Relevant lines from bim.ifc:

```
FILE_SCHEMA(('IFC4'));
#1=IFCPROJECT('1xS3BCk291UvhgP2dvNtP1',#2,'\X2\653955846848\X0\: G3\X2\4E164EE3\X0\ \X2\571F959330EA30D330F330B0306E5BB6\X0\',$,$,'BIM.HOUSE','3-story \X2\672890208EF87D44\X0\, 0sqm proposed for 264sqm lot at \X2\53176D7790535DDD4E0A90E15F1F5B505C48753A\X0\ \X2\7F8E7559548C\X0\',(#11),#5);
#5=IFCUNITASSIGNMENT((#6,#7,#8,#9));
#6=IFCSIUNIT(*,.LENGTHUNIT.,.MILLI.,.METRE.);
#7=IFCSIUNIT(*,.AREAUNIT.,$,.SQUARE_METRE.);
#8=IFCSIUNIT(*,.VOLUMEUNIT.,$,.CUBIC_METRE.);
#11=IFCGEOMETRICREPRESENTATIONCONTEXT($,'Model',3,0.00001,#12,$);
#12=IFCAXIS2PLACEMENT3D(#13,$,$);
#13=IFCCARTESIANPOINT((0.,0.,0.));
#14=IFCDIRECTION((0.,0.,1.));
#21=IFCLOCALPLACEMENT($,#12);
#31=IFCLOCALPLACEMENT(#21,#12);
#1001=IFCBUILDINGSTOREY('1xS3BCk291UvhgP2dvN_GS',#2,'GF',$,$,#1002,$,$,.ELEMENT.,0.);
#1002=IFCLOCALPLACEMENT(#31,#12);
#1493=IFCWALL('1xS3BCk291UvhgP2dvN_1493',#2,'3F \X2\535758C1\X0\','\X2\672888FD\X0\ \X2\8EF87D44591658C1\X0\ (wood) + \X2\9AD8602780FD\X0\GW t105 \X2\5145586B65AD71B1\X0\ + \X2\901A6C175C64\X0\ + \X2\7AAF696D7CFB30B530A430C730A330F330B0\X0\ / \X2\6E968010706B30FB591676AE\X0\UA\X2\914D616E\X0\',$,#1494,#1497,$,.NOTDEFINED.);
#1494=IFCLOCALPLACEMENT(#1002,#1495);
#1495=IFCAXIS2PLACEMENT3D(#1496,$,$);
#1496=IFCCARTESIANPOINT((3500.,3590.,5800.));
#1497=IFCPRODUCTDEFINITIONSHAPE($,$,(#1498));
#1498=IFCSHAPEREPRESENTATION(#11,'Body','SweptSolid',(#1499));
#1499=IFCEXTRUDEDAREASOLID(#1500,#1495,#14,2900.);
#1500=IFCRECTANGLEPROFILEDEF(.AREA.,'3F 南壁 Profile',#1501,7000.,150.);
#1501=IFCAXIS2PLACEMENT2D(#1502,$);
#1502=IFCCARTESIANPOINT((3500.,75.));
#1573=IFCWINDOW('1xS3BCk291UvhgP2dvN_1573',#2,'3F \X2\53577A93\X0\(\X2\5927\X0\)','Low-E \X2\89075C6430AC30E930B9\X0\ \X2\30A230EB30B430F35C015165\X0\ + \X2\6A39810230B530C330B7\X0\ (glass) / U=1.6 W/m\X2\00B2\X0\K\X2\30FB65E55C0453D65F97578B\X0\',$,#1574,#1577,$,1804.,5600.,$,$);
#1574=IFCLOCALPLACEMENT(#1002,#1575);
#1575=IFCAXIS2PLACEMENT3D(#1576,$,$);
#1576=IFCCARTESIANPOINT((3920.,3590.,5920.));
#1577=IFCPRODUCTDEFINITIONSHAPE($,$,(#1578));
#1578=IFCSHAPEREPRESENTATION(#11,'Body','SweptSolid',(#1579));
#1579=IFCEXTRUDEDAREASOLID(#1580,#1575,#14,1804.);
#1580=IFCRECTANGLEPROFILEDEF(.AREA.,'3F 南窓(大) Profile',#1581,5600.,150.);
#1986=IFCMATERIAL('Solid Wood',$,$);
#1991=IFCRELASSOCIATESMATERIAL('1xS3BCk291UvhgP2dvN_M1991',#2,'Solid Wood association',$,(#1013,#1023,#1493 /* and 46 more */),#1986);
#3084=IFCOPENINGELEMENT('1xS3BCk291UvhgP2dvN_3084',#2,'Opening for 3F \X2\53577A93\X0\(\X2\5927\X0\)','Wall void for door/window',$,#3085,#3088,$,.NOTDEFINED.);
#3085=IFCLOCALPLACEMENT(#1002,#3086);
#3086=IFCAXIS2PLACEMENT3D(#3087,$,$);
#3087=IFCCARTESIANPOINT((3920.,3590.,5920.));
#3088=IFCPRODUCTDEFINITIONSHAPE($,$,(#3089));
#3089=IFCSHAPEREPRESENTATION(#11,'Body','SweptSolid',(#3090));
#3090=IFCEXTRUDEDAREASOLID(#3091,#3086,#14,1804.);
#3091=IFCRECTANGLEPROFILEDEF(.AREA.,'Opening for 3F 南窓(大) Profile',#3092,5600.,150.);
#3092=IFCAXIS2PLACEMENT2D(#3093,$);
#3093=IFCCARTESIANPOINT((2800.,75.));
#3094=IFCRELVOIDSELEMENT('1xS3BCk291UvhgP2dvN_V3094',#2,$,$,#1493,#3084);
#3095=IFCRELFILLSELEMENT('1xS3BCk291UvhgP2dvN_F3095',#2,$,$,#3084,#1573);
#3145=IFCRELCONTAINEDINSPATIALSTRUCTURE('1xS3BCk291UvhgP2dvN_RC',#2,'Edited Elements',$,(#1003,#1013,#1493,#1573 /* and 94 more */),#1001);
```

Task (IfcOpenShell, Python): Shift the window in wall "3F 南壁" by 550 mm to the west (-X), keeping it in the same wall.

```python
import ifcopenshell
import ifcopenshell.api.geometry
import ifcopenshell.util.placement

model = ifcopenshell.open("bim.ifc")

window = model.by_guid("1xS3BCk291UvhgP2dvN_1573")
opening = window.FillsVoids[0].RelatingOpeningElement
wall = opening.VoidsElements[0].RelatingBuildingElement

wall_matrix = ifcopenshell.util.placement.get_local_placement(wall.ObjectPlacement)
shift = wall_matrix[:3, 0] * -550.0
before = ifcopenshell.util.placement.get_local_placement(window.ObjectPlacement)[:3, 3].copy()

# The window is not placed relative to its opening, so move both.
for product in (opening, window):
    matrix = ifcopenshell.util.placement.get_local_placement(product.ObjectPlacement)
    matrix[:3, 3] += shift
    ifcopenshell.api.geometry.edit_object_placement(model, product=product, matrix=matrix, is_si=False)

after = ifcopenshell.util.placement.get_local_placement(window.ObjectPlacement)[:3, 3]
print("window moved by", (after - before).round(3) + 0.0)

model.write("bim-out.ifc")
```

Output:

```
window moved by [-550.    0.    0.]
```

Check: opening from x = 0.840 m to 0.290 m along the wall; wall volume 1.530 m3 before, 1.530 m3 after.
